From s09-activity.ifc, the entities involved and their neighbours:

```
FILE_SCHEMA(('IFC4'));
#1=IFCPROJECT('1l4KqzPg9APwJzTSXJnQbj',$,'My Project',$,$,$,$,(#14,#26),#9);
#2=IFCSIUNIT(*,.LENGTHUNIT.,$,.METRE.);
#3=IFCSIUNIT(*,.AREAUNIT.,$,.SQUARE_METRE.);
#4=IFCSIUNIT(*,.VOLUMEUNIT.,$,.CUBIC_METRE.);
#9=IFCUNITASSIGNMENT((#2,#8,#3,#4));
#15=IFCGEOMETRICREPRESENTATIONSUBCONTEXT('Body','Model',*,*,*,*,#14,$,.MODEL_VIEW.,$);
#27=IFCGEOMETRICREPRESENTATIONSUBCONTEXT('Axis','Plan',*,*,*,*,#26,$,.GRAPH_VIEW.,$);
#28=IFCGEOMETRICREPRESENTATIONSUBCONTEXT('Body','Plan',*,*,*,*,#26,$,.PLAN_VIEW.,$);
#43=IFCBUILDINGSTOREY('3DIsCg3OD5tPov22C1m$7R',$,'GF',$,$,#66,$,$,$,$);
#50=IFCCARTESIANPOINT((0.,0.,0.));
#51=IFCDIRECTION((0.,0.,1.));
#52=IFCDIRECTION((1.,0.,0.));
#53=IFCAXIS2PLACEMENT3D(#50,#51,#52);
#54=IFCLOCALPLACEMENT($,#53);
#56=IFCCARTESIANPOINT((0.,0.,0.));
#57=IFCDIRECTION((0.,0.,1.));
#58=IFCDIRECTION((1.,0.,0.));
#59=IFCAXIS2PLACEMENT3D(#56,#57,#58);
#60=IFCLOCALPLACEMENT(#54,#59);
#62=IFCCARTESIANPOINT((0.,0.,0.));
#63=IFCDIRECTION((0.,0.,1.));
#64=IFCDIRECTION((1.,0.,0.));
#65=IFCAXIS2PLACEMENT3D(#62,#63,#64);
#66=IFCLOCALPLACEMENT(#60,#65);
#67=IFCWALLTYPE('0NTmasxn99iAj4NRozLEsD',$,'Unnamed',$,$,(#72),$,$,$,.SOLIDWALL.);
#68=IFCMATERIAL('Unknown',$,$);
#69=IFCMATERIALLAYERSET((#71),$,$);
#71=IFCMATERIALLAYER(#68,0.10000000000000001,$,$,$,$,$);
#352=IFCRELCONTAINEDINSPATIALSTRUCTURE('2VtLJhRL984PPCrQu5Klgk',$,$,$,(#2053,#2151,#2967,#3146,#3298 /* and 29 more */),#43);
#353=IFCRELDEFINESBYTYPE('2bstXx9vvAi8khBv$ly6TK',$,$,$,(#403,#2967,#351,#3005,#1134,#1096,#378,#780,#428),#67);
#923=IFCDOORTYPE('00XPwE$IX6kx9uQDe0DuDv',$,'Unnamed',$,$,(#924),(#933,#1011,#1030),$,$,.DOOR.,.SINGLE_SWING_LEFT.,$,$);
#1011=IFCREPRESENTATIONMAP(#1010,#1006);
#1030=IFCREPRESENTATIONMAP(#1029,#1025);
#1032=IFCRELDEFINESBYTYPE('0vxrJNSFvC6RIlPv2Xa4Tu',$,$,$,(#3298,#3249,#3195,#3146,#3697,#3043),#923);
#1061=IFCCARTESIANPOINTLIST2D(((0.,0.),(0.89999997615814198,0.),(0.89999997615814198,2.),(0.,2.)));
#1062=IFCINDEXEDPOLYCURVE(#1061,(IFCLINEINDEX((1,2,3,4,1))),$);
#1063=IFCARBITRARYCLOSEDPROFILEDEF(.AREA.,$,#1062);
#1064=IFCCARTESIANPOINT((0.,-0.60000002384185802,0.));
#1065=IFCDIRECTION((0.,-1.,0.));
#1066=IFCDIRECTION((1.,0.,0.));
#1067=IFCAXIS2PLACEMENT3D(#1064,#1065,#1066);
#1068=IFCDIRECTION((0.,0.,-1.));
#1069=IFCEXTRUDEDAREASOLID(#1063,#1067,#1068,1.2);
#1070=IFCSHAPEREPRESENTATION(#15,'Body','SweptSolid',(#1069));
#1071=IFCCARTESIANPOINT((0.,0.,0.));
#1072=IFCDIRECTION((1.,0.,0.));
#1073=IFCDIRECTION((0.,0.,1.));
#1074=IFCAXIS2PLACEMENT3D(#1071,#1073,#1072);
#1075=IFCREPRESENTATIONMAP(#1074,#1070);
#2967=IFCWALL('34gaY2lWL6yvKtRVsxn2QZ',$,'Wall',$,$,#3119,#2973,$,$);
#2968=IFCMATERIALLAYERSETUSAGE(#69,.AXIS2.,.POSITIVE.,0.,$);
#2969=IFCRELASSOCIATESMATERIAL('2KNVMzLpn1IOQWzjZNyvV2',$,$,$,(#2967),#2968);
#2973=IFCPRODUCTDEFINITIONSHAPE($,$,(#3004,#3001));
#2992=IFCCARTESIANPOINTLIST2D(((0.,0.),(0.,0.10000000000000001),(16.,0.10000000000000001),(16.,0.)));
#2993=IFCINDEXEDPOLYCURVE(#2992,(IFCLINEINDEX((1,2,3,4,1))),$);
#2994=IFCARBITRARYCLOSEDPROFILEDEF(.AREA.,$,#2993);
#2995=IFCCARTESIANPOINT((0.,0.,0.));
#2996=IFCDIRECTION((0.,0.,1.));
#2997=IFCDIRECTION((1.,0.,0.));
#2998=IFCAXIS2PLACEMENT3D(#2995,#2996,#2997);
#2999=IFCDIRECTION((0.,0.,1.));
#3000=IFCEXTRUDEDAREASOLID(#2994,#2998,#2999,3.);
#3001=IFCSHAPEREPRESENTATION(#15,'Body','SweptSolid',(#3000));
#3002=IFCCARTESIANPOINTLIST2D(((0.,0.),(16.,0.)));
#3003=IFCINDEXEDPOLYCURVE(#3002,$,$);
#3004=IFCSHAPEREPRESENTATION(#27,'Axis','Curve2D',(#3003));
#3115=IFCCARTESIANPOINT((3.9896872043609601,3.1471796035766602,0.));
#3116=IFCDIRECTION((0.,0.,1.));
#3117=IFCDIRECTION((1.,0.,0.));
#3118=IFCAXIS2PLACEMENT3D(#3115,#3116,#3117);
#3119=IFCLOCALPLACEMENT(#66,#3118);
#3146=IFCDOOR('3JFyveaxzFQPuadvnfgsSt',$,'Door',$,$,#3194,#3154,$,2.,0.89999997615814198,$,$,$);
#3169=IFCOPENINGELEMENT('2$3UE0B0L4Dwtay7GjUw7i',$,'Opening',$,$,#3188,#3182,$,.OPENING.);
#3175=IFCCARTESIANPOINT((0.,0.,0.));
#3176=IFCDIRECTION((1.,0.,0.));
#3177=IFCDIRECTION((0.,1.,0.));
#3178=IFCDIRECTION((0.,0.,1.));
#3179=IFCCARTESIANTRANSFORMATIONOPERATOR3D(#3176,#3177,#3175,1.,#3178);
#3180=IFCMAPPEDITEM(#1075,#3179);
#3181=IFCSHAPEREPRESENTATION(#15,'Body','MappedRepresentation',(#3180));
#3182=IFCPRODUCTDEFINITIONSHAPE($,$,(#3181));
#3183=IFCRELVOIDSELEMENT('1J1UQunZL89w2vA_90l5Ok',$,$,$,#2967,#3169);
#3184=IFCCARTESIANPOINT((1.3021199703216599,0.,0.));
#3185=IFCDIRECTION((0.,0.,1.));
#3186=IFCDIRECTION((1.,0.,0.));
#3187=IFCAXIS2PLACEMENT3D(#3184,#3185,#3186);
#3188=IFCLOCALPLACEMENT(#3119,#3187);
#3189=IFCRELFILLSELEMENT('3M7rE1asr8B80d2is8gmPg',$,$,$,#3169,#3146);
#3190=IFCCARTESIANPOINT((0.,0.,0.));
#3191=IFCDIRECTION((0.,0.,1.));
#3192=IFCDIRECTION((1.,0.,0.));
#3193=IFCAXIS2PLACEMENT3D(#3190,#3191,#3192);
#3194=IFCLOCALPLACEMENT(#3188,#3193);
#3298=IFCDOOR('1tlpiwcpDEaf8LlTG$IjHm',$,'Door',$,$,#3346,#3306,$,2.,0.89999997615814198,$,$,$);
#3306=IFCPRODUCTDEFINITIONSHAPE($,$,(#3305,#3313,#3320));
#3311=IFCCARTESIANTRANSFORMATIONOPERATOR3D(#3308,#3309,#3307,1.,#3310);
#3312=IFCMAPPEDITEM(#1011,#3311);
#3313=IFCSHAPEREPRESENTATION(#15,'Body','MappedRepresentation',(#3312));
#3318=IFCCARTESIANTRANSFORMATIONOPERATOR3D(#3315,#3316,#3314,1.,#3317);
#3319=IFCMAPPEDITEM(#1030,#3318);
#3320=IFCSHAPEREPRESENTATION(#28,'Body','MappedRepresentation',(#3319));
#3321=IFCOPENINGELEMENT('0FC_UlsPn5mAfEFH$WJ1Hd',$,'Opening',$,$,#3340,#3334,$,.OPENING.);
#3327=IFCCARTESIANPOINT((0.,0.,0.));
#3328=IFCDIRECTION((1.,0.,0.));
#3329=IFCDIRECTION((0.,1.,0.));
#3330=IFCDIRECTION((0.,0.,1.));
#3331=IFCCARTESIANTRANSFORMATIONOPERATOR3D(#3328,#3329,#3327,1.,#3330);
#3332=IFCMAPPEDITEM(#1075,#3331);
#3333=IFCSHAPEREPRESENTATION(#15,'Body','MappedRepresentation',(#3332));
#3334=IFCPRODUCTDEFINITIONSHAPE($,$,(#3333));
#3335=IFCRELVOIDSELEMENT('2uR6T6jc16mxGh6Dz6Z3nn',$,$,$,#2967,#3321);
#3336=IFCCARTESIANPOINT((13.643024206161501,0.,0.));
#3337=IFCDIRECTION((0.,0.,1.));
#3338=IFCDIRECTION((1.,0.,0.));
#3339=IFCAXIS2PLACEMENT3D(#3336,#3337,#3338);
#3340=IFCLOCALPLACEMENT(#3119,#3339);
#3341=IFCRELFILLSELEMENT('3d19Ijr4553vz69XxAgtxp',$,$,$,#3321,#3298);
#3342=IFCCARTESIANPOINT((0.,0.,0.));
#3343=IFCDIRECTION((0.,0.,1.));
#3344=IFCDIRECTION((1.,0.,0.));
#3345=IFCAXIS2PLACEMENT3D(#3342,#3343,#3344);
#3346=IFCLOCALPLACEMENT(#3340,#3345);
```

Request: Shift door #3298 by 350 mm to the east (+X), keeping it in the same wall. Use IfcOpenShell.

```python
import ifcopenshell
import ifcopenshell.api.geometry
import ifcopenshell.util.placement

model = ifcopenshell.open("s09-activity.ifc")

door = model.by_guid("1tlpiwcpDEaf8LlTG$IjHm")
opening = door.FillsVoids[0].RelatingOpeningElement
wall = opening.VoidsElements[0].RelatingBuildingElement

wall_matrix = ifcopenshell.util.placement.get_local_placement(wall.ObjectPlacement)
shift = wall_matrix[:3, 0] * 0.35
before = ifcopenshell.util.placement.get_local_placement(door.ObjectPlacement)[:3, 3].copy()

# The door is placed relative to its opening, so it follows when the opening moves.
matrix = ifcopenshell.util.placement.get_local_placement(opening.ObjectPlacement)
matrix[:3, 3] += shift
ifcopenshell.api.geometry.edit_object_placement(
    model, product=opening, matrix=matrix, is_si=False, should_transform_children=True
)

after = ifcopenshell.util.placement.get_local_placement(door.ObjectPlacement)[:3, 3]
print("door moved by", (after - before).round(3) + 0.0)

model.write("s09-activity_edited.ifc")
```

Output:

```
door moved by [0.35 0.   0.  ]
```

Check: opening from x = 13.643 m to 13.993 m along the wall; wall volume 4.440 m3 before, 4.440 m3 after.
